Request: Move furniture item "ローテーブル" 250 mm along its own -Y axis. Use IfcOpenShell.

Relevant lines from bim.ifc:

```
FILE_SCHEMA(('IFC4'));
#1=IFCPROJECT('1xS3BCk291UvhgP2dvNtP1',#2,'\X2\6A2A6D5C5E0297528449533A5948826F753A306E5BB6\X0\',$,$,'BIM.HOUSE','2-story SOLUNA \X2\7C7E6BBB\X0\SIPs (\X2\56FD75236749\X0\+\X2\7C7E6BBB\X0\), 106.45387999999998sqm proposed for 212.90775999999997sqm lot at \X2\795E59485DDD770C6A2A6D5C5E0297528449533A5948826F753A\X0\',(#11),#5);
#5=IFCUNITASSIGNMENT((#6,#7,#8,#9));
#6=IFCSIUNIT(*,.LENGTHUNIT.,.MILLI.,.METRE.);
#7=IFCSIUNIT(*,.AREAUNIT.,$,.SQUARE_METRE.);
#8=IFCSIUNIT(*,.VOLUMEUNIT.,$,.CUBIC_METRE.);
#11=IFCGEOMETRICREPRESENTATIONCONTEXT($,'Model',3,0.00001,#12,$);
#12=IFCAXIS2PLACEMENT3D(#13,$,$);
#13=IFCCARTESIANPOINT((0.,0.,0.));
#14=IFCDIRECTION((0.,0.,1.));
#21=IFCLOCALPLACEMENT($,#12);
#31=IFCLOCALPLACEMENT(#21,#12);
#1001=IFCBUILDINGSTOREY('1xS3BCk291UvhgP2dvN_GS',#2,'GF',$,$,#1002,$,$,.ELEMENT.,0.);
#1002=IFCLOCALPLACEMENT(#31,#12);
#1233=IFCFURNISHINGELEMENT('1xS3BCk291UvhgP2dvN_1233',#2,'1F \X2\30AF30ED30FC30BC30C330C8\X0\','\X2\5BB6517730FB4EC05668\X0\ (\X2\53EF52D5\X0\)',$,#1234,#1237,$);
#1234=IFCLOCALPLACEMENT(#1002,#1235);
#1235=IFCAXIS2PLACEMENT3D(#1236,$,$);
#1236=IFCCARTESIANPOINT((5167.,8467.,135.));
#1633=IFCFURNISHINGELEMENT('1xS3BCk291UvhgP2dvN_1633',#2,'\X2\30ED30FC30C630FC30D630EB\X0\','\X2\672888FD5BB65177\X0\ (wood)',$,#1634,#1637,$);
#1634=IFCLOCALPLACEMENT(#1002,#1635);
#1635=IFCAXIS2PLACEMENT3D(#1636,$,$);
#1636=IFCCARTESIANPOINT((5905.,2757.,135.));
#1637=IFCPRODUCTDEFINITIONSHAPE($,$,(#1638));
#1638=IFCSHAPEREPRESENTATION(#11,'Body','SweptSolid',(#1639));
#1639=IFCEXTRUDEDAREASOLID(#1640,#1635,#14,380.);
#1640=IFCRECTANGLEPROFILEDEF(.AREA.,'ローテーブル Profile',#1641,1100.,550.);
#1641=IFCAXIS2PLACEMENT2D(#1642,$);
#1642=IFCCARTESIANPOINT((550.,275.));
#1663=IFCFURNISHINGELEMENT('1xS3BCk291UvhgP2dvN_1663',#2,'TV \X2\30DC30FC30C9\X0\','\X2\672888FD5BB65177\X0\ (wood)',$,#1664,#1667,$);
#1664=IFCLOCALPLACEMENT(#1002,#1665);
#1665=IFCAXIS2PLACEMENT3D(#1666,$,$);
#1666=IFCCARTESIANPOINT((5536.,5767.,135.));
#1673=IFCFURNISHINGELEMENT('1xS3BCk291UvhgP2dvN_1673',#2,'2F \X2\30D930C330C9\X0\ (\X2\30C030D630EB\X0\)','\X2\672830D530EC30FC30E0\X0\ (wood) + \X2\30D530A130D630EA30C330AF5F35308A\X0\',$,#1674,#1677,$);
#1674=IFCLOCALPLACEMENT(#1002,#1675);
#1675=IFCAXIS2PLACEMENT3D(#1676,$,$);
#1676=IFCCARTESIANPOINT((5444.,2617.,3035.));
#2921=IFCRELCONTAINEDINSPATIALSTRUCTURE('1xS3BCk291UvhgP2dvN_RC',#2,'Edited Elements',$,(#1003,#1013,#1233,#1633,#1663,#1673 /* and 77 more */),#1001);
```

```python
import ifcopenshell
import ifcopenshell.api.geometry
import ifcopenshell.util.placement
import ifcopenshell.util.unit

model = ifcopenshell.open("bim.ifc")
unit_scale = ifcopenshell.util.unit.calculate_unit_scale(model)

item = model.by_guid("1xS3BCk291UvhgP2dvN_1633")
matrix = ifcopenshell.util.placement.get_local_placement(item.ObjectPlacement)
matrix[:3, 3] -= matrix[:3, 1] * 0.25 / unit_scale
ifcopenshell.api.geometry.edit_object_placement(model, product=item, matrix=matrix, is_si=False)

print(ifcopenshell.util.placement.get_local_placement(item.ObjectPlacement).round(3) + 0.0)

model.write("bim_updated.ifc")
```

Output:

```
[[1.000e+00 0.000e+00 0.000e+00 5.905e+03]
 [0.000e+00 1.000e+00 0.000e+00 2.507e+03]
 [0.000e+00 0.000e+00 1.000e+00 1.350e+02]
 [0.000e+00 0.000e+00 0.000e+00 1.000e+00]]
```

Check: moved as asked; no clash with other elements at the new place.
